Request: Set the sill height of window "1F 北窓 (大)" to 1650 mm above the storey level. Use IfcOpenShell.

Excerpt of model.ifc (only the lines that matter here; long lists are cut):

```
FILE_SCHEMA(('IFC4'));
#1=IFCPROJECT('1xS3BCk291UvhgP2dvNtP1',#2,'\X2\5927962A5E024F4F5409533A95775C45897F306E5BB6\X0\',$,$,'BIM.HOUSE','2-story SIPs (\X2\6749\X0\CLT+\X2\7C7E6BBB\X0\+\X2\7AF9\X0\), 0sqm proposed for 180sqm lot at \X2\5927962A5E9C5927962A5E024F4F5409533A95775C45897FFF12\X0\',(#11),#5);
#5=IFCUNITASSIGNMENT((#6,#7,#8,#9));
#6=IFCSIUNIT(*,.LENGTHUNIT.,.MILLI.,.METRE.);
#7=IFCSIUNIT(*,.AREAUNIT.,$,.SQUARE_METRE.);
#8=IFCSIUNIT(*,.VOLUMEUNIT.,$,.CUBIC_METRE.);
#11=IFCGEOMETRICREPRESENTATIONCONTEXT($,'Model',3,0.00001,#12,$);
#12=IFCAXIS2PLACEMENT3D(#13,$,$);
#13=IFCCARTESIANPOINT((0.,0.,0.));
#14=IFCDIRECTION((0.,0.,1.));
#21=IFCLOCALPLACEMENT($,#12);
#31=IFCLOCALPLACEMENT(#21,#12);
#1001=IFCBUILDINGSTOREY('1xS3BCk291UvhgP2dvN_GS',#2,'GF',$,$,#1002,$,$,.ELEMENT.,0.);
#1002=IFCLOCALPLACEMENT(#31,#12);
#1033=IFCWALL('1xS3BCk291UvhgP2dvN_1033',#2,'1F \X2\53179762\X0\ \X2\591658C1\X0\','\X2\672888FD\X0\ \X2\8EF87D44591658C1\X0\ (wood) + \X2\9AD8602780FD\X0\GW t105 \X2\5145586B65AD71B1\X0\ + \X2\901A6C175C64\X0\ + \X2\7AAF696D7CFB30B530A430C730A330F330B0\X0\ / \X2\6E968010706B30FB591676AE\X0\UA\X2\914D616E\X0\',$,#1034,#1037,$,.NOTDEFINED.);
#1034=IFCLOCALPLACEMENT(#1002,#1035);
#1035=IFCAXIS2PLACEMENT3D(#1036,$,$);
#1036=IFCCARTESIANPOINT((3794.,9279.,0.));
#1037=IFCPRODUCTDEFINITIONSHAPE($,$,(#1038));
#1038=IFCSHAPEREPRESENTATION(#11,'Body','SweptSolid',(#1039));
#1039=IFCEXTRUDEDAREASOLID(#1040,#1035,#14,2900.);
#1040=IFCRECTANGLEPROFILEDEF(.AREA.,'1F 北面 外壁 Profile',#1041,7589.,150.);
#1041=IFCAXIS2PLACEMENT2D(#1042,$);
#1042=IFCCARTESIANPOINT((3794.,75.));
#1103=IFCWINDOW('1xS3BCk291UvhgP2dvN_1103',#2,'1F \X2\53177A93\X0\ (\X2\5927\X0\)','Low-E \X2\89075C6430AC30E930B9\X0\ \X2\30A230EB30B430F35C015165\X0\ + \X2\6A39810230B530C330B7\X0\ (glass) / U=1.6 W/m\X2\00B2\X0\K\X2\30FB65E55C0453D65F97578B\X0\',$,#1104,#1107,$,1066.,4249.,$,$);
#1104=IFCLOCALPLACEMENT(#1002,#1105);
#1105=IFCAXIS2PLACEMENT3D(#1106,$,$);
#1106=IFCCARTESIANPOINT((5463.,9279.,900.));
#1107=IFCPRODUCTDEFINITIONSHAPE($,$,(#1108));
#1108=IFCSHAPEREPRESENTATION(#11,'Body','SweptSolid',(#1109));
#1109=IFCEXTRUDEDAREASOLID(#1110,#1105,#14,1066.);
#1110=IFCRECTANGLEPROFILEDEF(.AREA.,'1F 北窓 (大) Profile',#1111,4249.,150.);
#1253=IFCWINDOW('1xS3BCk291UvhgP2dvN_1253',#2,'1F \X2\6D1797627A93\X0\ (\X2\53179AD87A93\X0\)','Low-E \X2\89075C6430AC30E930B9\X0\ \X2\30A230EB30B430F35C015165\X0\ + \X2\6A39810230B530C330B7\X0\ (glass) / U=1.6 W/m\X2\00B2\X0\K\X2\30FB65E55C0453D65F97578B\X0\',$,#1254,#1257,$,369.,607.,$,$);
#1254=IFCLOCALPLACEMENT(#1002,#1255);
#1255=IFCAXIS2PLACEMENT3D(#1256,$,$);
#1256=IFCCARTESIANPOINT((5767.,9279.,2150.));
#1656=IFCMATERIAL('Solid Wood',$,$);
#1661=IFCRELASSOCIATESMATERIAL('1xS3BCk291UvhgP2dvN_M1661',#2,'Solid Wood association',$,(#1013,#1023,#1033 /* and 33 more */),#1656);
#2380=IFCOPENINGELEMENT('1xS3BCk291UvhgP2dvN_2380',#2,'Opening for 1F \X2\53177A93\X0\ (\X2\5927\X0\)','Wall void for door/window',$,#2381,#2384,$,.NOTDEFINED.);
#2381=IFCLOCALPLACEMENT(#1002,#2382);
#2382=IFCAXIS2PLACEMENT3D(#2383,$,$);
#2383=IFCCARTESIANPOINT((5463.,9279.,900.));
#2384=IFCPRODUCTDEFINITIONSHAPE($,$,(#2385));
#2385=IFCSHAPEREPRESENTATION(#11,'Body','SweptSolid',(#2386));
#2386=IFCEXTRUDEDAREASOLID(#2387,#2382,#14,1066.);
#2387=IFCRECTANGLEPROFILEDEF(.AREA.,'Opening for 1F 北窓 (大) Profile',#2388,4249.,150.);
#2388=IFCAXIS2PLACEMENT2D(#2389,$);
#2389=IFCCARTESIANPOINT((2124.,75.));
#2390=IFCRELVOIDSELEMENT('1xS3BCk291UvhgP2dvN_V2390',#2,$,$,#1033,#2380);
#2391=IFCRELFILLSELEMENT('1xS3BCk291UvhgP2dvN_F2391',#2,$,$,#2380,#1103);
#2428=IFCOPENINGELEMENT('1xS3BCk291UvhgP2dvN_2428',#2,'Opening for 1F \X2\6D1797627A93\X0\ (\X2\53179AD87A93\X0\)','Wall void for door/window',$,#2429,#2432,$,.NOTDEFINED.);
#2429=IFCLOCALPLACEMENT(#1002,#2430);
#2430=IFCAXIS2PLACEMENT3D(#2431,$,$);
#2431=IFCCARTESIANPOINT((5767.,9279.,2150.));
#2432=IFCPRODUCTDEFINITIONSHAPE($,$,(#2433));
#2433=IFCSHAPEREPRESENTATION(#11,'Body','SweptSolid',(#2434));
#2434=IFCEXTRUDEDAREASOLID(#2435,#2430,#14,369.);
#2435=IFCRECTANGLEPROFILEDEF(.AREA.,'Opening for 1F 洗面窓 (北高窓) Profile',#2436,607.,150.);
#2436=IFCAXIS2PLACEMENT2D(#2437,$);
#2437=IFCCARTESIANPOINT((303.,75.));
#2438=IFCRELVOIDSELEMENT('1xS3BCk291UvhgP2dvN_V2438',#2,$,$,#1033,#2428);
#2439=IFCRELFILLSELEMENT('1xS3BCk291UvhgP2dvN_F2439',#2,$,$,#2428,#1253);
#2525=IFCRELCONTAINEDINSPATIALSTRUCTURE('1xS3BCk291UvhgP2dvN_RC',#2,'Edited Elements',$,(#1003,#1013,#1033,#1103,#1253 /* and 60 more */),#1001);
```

```python
import numpy as np
import ifcopenshell
import ifcopenshell.api.geometry
import ifcopenshell.geom
import ifcopenshell.util.element
import ifcopenshell.util.placement
import ifcopenshell.util.shape
import ifcopenshell.util.unit

model = ifcopenshell.open("model.ifc")
unit_scale = ifcopenshell.util.unit.calculate_unit_scale(model)

window = model.by_guid("1xS3BCk291UvhgP2dvN_1103")
opening = window.FillsVoids[0].RelatingOpeningElement
storey = ifcopenshell.util.element.get_container(window, ifc_class="IfcBuildingStorey")
level = ifcopenshell.util.placement.get_local_placement(storey.ObjectPlacement)[2, 3]

# The opening's origin need not be at the sill, so measure its lowest point.
shape = ifcopenshell.geom.create_shape(ifcopenshell.geom.settings(), opening)
bottom = ifcopenshell.util.shape.get_shape_bottom_elevation(shape, shape.geometry) / unit_scale
dz = level + 1.65 / unit_scale - bottom

shift = np.array([0.0, 0.0, dz])
# The window is not placed relative to its opening, so move both.
for product in (opening, window):
    matrix = ifcopenshell.util.placement.get_local_placement(product.ObjectPlacement)
    matrix[:3, 3] += shift
    ifcopenshell.api.geometry.edit_object_placement(model, product=product, matrix=matrix, is_si=False)

print(f"moved by {dz * unit_scale:+.3f} m")

model.write("model-out.ifc")
```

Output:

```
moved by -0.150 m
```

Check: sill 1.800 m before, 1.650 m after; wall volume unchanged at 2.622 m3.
